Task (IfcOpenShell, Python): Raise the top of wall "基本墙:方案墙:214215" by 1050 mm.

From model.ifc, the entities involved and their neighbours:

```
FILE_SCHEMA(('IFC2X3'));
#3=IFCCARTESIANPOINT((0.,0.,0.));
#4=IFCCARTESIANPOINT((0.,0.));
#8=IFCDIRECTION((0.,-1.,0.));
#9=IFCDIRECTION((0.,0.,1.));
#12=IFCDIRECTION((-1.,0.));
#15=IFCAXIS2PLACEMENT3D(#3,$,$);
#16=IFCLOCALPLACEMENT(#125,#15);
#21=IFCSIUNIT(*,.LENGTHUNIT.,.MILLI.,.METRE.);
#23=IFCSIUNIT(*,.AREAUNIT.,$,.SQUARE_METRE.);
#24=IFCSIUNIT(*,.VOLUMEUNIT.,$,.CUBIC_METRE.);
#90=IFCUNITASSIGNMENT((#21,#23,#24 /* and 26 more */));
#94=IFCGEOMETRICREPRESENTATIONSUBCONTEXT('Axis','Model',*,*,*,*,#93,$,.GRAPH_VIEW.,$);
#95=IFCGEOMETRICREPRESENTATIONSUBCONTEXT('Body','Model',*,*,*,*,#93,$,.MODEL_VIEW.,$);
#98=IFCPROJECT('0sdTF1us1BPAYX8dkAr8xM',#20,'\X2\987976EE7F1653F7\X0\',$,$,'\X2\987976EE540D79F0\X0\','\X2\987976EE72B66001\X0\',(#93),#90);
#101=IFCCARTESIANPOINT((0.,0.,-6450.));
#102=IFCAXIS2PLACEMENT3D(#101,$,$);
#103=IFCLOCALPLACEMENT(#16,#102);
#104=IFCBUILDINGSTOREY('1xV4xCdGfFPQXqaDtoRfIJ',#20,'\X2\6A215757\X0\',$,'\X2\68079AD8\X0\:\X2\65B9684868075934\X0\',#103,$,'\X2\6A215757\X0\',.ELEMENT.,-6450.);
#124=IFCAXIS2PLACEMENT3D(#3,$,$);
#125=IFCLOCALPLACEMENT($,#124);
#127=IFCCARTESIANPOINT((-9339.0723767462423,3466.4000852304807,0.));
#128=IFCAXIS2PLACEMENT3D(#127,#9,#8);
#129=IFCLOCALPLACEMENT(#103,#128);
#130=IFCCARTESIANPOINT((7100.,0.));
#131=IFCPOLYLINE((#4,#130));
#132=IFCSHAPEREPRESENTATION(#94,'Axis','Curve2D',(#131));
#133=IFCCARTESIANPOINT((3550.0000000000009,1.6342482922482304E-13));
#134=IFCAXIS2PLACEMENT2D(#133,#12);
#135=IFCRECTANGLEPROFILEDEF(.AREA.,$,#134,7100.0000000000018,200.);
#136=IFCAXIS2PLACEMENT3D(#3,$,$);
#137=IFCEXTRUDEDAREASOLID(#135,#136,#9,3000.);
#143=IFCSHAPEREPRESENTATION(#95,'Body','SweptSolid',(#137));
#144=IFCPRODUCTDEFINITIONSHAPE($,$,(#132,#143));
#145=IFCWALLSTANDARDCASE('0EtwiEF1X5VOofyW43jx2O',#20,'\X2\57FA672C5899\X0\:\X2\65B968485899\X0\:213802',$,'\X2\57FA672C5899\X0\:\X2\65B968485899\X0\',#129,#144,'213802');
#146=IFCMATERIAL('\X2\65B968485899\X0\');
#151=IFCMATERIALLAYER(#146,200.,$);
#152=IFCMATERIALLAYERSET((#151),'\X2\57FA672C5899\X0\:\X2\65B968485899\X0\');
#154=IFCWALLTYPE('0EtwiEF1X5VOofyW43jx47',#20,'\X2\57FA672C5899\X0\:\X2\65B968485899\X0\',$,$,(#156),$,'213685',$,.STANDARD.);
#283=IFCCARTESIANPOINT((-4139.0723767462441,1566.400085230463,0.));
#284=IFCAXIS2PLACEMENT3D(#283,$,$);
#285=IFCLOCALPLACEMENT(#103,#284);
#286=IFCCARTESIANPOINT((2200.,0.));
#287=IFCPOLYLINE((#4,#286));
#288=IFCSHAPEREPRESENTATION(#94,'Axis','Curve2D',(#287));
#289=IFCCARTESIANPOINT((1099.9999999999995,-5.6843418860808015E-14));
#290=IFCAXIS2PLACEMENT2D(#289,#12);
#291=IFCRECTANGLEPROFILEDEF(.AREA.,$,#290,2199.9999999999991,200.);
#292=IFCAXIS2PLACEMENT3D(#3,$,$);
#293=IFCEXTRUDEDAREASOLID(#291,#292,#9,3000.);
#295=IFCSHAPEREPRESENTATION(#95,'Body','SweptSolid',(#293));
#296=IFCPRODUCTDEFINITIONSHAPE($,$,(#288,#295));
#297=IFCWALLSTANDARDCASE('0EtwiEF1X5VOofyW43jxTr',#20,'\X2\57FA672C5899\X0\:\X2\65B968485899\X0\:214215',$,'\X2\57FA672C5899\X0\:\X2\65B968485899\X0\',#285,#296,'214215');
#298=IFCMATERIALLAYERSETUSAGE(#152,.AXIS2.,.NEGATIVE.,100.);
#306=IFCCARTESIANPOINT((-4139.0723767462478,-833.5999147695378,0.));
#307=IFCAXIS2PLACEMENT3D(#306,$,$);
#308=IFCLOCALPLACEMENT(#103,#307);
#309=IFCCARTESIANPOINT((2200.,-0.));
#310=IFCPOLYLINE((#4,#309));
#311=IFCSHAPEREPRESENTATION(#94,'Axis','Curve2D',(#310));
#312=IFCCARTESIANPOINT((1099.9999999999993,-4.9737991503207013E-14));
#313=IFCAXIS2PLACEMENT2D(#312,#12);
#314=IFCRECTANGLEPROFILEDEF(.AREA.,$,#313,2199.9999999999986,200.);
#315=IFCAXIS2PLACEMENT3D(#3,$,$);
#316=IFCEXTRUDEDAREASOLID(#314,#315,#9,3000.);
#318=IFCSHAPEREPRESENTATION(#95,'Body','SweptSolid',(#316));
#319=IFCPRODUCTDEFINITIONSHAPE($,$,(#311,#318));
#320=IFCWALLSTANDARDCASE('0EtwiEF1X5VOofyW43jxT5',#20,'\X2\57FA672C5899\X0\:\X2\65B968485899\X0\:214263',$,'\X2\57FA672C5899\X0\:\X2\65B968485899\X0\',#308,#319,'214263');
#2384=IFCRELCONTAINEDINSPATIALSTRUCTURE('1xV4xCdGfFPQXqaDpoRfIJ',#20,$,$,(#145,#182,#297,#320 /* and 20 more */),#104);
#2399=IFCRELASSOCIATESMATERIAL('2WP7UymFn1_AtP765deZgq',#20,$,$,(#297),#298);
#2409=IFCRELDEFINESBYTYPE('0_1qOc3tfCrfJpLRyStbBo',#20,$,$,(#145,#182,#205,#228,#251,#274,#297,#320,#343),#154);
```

```python
import ifcopenshell
import ifcopenshell.geom
import ifcopenshell.util.representation
import ifcopenshell.util.shape
import ifcopenshell.util.unit

model = ifcopenshell.open("model.ifc")
unit_scale = ifcopenshell.util.unit.calculate_unit_scale(model)
settings = ifcopenshell.geom.settings()


def volume(element):
    """Net volume in cubic metres, openings subtracted."""
    shape = ifcopenshell.geom.create_shape(settings, element)
    return ifcopenshell.util.shape.get_volume(shape.geometry)


wall = model.by_id(297)
before = volume(wall)

body = ifcopenshell.util.representation.get_representation(wall, "Model", "Body")
solid = body.Items[0]
old_height = solid.Depth
solid.Depth += 1.05 / unit_scale
after = volume(wall)

print(f"height {old_height:g} -> {solid.Depth:g}, volume {before:.3f} -> {after:.3f} m3")

model.write("model_rev.ifc")
```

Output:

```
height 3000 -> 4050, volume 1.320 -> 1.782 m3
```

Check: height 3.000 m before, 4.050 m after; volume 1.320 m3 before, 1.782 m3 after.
